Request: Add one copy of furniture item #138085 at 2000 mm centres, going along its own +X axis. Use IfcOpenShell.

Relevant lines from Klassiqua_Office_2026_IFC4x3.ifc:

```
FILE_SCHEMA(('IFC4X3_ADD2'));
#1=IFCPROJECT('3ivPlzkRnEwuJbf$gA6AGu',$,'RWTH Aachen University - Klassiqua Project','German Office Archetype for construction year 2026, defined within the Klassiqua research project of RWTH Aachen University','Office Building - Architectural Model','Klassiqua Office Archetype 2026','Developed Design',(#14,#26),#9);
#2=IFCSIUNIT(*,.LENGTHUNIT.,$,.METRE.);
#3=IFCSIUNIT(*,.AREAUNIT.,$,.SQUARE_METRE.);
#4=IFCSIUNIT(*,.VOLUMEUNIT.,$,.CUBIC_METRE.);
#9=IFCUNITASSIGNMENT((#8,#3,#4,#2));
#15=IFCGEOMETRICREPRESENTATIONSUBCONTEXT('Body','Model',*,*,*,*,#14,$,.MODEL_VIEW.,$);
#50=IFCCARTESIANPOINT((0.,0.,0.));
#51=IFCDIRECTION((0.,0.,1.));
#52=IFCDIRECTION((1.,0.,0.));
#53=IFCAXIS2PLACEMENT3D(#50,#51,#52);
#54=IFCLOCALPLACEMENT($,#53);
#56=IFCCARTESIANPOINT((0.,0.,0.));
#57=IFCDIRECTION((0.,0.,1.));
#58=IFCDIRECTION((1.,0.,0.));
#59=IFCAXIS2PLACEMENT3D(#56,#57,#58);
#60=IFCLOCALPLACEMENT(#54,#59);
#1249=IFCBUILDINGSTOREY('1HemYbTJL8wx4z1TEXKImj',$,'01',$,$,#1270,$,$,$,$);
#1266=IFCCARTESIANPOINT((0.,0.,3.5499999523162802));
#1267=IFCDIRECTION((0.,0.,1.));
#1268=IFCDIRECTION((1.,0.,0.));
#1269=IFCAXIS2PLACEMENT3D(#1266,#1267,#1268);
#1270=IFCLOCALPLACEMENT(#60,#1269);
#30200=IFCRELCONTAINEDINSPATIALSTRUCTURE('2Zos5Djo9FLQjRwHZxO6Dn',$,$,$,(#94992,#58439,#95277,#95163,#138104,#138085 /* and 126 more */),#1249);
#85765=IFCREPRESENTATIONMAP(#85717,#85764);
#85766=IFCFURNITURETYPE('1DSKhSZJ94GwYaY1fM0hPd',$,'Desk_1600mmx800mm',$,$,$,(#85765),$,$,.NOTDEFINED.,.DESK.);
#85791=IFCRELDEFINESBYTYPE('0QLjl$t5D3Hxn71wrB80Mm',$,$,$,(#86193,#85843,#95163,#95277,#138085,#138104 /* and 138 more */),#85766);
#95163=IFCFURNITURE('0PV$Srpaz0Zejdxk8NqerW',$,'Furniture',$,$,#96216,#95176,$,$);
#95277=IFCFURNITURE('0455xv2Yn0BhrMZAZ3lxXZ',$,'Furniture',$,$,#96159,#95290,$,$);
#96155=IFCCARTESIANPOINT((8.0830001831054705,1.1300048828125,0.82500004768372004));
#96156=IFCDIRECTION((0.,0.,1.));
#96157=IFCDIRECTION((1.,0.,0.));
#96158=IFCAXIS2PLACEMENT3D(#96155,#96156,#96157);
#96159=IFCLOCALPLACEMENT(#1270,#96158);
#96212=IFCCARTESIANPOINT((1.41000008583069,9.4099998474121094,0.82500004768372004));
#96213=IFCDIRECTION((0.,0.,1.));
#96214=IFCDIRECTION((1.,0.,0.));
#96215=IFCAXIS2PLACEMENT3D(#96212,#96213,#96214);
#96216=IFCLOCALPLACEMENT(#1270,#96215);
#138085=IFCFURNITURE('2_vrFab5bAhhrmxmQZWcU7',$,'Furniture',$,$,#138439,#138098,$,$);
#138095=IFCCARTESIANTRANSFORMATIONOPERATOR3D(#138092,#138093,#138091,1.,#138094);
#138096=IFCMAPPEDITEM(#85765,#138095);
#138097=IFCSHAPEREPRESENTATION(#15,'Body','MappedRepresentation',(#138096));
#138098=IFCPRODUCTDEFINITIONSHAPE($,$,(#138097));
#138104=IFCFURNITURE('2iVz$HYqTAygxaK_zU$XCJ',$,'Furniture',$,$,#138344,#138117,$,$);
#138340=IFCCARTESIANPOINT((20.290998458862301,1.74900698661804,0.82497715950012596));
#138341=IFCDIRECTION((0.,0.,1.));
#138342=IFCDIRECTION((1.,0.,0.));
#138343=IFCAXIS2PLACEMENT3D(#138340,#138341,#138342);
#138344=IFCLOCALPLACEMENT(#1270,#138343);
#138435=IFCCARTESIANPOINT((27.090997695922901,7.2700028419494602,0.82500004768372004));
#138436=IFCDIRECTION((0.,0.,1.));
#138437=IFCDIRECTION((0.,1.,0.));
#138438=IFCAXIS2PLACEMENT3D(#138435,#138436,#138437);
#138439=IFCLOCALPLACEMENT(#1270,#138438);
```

```python
import ifcopenshell
import ifcopenshell.api.geometry
import ifcopenshell.api.root
import ifcopenshell.util.element
import ifcopenshell.util.placement
import ifcopenshell.util.unit

model = ifcopenshell.open("Klassiqua_Office_2026_IFC4x3.ifc")
unit_scale = ifcopenshell.util.unit.calculate_unit_scale(model)

source = model.by_id(138085)
base = ifcopenshell.util.placement.get_local_placement(source.ObjectPlacement)
step = base[:3, 0] * 2 / unit_scale

for i in range(1, 2):
    copy = ifcopenshell.api.root.copy_class(model, product=source)
    copy.Representation = ifcopenshell.util.element.copy_deep(
        model, source.Representation, exclude=["IfcGeometricRepresentationContext", "IfcRepresentationMap"]
    )
    matrix = base.copy()
    matrix[:3, 3] += i * step
    print("added at", matrix[:3, 3].round(3) + 0.0)
    ifcopenshell.api.geometry.edit_object_placement(model, product=copy, matrix=matrix, is_si=False)

model.write("Klassiqua_Office_2026_IFC4x3_edited.ifc")
```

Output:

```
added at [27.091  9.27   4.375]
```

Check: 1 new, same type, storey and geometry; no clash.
